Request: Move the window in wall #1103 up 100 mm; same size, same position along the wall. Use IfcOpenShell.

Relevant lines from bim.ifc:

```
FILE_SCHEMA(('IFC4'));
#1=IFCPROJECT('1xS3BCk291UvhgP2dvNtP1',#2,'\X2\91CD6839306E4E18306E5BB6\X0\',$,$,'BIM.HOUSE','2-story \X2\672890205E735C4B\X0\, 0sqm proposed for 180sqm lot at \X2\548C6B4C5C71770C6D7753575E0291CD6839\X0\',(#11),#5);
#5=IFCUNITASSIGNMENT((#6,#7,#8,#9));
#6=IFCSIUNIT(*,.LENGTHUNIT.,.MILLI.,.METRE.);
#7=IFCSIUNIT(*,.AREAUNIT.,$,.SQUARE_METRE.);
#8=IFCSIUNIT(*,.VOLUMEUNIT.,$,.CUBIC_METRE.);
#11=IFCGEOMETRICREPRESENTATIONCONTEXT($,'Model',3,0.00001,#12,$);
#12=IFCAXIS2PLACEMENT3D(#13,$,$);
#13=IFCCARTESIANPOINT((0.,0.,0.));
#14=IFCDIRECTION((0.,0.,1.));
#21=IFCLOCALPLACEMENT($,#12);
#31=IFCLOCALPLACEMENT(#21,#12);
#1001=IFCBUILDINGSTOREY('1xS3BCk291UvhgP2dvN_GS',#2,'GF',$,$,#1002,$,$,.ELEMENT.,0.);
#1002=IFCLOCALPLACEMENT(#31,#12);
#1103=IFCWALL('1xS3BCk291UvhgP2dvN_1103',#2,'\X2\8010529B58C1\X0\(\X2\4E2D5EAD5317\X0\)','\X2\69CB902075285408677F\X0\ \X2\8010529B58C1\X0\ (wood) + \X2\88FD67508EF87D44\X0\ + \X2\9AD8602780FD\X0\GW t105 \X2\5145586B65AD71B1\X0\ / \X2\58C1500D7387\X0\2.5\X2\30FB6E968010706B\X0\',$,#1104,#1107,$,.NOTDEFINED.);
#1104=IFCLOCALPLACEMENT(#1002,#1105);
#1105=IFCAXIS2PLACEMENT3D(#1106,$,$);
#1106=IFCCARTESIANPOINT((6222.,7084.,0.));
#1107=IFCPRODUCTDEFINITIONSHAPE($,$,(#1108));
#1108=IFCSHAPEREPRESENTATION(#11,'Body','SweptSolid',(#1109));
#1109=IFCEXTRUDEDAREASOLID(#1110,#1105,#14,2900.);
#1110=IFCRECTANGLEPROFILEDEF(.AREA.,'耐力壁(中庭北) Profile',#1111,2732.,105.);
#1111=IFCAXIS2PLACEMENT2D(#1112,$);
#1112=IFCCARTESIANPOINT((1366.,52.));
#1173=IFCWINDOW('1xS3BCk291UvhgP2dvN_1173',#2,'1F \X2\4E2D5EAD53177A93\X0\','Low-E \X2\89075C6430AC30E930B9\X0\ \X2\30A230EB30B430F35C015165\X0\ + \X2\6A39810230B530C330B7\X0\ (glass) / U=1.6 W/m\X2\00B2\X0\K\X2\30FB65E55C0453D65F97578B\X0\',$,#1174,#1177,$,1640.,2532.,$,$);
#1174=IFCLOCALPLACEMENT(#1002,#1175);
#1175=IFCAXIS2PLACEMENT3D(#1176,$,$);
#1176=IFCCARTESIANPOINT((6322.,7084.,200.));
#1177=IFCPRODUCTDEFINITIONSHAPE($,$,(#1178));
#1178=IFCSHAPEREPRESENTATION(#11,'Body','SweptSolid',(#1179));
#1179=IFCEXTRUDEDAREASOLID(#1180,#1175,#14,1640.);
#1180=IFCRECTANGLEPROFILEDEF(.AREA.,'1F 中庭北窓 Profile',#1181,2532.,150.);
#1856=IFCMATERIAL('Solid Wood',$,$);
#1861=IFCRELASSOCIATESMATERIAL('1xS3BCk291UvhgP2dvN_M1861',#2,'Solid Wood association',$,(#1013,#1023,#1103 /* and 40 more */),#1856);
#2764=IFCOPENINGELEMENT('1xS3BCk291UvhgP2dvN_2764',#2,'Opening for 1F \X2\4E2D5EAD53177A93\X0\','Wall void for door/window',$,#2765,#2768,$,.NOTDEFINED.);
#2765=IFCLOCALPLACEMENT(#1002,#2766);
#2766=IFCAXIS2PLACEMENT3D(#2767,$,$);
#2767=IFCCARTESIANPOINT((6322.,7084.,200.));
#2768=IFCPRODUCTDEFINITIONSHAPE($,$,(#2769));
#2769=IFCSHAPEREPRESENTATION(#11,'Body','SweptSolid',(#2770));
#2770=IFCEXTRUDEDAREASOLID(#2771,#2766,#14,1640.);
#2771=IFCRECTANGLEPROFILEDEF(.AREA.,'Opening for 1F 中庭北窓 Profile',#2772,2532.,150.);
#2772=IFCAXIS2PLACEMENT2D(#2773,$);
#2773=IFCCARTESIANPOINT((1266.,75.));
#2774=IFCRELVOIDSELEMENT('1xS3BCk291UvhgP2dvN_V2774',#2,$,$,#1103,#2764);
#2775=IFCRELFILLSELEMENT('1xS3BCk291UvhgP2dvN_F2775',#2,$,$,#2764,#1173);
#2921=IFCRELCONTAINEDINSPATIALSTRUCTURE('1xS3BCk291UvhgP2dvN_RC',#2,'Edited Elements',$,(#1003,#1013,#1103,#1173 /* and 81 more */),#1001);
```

```python
import numpy as np
import ifcopenshell
import ifcopenshell.api.geometry
import ifcopenshell.util.placement
import ifcopenshell.util.unit

model = ifcopenshell.open("bim.ifc")
unit_scale = ifcopenshell.util.unit.calculate_unit_scale(model)

window = model.by_id(1173)
opening = window.FillsVoids[0].RelatingOpeningElement
dz = 0.1 / unit_scale

shift = np.array([0.0, 0.0, dz])
# The window is not placed relative to its opening, so move both.
for product in (opening, window):
    matrix = ifcopenshell.util.placement.get_local_placement(product.ObjectPlacement)
    matrix[:3, 3] += shift
    ifcopenshell.api.geometry.edit_object_placement(model, product=product, matrix=matrix, is_si=False)

print(f"moved by {dz * unit_scale:+.3f} m")

model.write("bim_updated.ifc")
```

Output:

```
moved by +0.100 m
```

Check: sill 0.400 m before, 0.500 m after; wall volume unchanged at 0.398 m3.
